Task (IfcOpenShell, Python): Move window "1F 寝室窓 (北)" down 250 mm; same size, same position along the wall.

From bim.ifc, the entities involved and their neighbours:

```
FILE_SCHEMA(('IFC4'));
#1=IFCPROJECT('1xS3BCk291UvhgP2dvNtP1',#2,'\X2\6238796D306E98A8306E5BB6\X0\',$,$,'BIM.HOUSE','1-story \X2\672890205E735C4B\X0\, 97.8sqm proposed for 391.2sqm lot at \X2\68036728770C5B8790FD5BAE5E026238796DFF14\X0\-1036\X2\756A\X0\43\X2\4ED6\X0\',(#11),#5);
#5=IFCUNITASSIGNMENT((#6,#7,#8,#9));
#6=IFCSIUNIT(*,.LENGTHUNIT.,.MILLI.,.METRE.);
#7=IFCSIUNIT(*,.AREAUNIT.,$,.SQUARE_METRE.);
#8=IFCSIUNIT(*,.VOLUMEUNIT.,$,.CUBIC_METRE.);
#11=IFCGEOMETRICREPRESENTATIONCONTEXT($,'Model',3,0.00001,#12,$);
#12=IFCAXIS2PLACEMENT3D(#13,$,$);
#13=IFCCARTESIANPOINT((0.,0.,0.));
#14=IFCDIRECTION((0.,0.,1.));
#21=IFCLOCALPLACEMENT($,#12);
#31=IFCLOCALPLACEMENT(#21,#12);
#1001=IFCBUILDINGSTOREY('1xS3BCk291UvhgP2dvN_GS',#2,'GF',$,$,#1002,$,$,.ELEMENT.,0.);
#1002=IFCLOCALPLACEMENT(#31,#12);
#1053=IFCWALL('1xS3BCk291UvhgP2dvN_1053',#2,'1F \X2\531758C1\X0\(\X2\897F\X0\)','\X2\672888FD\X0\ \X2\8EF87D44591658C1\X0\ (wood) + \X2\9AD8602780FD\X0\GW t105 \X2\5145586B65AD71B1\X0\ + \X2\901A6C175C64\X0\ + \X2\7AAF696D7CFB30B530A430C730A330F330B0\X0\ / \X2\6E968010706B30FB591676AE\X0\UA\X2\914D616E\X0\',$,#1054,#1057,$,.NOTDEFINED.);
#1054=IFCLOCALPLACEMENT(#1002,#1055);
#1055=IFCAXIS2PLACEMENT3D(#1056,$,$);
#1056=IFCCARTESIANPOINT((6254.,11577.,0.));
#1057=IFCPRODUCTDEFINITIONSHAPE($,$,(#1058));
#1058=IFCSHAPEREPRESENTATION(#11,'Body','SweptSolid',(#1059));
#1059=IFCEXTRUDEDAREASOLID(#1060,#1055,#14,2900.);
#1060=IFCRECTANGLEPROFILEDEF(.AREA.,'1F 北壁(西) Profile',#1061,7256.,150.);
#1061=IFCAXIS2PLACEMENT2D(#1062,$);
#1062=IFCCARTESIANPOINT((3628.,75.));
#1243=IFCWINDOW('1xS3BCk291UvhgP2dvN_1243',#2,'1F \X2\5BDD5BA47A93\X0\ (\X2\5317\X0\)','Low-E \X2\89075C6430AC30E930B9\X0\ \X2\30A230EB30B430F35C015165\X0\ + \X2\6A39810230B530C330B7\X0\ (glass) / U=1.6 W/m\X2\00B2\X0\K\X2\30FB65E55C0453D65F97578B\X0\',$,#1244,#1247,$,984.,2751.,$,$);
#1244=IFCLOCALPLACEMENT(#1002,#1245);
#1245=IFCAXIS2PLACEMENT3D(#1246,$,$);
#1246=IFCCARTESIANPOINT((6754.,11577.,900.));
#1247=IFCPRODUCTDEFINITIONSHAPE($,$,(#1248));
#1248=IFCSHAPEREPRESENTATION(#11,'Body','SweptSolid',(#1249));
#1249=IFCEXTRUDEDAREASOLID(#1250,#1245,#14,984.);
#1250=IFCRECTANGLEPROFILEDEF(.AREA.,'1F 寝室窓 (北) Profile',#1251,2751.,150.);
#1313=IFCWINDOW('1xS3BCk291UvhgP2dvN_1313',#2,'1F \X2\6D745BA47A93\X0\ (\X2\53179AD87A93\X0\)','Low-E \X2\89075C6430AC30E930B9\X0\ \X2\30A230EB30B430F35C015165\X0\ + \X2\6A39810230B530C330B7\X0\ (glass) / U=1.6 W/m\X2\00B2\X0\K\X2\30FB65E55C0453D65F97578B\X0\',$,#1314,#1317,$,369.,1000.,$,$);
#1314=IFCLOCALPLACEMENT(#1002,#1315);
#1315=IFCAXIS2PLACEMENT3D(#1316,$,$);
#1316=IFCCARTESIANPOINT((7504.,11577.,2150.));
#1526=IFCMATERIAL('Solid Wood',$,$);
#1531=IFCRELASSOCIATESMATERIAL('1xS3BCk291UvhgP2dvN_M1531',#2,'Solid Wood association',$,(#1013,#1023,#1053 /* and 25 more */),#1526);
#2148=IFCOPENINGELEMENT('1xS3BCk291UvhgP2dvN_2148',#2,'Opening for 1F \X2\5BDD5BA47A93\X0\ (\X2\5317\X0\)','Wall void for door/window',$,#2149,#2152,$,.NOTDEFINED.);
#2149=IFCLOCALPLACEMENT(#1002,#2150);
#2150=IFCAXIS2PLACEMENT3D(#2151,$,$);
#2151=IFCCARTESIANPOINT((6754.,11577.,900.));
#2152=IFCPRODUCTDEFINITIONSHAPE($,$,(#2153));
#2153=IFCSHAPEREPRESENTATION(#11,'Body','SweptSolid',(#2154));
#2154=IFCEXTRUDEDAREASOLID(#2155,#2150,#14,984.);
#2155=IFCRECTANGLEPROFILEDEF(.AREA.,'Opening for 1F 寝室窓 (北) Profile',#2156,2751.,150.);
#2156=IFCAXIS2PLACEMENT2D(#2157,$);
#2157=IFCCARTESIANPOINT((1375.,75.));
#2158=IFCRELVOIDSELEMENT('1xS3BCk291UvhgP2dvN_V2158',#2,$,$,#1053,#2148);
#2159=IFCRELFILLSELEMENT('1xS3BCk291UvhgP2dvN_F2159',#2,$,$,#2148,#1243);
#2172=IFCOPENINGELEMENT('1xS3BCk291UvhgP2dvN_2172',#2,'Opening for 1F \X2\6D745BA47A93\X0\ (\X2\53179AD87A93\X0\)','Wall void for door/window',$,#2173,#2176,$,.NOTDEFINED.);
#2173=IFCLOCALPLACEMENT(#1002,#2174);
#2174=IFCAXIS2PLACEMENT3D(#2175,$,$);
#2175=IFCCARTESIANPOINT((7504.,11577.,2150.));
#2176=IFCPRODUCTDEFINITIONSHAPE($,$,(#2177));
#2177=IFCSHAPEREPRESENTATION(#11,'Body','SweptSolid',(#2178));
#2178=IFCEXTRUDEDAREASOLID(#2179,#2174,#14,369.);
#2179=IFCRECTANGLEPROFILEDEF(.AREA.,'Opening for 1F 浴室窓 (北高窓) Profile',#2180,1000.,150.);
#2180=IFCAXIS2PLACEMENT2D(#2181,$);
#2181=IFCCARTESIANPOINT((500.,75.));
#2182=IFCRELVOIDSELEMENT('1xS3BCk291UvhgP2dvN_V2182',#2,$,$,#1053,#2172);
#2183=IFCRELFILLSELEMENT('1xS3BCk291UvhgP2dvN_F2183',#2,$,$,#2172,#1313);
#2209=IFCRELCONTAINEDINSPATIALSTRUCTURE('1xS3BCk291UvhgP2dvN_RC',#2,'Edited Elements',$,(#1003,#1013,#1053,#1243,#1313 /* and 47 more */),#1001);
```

```python
import numpy as np
import ifcopenshell
import ifcopenshell.api.geometry
import ifcopenshell.util.placement
import ifcopenshell.util.unit

model = ifcopenshell.open("bim.ifc")
unit_scale = ifcopenshell.util.unit.calculate_unit_scale(model)

window = model.by_guid("1xS3BCk291UvhgP2dvN_1243")
opening = window.FillsVoids[0].RelatingOpeningElement
dz = -250.0

shift = np.array([0.0, 0.0, dz])
# The window is not placed relative to its opening, so move both.
for product in (opening, window):
    matrix = ifcopenshell.util.placement.get_local_placement(product.ObjectPlacement)
    matrix[:3, 3] += shift
    ifcopenshell.api.geometry.edit_object_placement(model, product=product, matrix=matrix, is_si=False)

print(f"moved by {dz * unit_scale:+.3f} m")

model.write("bim_v2.ifc")
```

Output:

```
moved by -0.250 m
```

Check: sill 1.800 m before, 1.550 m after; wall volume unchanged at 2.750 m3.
